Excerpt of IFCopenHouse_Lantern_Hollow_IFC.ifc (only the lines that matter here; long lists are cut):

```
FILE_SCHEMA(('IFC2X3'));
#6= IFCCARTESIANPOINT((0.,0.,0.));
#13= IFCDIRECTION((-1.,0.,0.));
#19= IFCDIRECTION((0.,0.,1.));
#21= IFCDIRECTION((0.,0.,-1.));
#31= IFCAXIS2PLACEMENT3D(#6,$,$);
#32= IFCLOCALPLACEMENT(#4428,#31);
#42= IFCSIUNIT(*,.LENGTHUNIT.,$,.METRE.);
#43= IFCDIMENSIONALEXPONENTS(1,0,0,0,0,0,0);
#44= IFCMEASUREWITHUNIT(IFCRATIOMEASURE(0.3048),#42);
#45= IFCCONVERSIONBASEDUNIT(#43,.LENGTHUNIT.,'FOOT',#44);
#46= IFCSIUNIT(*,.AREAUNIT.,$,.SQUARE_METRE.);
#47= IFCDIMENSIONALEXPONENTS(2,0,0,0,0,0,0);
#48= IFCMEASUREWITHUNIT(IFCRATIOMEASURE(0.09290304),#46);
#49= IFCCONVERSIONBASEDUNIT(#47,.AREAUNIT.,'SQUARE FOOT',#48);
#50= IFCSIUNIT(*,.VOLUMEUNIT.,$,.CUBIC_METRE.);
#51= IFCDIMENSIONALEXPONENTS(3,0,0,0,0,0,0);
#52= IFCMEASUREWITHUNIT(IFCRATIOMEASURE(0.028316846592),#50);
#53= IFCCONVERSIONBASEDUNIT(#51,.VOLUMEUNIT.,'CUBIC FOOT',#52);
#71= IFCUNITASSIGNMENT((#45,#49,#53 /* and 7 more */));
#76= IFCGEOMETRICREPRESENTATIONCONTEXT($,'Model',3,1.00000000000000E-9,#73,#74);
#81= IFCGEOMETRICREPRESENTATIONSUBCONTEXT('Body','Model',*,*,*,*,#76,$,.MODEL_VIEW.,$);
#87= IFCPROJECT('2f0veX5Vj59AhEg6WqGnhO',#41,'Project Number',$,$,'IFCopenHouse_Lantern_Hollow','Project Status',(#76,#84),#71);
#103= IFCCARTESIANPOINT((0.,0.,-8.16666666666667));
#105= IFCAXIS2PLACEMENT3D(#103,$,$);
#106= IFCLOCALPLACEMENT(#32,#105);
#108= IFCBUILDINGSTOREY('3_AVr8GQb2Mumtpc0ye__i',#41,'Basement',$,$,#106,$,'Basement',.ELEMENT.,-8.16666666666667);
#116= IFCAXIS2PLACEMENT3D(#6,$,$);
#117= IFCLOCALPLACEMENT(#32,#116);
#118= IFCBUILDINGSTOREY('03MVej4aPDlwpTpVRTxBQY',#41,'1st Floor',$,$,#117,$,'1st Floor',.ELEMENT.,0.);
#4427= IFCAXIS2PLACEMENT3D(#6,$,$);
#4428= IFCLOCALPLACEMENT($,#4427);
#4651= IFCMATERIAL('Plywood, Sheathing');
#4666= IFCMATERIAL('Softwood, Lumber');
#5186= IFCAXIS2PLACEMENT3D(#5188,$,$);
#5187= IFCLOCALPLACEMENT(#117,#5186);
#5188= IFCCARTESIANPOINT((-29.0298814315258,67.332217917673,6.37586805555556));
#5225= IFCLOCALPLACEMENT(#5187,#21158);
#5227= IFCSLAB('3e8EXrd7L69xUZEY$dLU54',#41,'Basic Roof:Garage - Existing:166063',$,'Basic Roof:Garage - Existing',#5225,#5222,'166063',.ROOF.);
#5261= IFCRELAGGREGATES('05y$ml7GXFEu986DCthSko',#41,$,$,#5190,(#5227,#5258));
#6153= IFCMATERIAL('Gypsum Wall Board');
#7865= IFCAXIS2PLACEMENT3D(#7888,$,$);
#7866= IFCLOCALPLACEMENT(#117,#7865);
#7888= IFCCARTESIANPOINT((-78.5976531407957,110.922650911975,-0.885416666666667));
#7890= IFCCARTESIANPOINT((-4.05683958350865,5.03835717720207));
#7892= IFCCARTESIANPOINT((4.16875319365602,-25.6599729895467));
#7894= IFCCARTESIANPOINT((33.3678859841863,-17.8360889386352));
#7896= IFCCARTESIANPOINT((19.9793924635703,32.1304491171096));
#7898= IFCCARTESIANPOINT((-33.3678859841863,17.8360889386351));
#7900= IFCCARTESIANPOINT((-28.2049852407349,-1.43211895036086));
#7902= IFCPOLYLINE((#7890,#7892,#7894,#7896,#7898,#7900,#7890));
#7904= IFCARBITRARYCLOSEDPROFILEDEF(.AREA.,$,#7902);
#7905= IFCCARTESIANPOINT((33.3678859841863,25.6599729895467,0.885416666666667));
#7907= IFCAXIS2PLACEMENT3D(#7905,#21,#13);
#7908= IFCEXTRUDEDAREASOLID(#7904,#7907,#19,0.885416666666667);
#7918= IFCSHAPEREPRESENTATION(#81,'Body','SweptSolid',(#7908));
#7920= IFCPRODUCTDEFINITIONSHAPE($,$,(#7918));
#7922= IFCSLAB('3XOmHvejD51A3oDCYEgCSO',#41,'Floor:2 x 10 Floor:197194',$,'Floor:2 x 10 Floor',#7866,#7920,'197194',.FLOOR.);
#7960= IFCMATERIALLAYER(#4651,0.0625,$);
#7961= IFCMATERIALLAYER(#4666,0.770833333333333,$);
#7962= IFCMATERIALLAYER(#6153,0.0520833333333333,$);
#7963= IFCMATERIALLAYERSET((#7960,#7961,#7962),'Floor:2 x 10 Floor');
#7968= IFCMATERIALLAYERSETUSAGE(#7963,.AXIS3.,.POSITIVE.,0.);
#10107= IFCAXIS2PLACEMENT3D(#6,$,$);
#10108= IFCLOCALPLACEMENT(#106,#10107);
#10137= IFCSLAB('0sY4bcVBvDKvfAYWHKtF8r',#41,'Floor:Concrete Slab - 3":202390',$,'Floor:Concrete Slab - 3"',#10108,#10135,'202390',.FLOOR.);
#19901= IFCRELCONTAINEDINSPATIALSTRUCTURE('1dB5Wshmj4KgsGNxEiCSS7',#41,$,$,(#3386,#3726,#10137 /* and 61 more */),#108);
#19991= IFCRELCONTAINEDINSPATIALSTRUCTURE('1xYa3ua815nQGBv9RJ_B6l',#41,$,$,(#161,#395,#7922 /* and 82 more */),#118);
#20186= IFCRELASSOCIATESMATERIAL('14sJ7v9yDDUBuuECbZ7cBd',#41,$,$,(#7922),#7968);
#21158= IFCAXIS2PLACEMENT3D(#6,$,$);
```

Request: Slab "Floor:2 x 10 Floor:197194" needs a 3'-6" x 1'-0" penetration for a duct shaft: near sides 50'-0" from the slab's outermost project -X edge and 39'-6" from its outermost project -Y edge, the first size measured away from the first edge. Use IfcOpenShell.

```python
import numpy as np
import ifcopenshell
import ifcopenshell.api.feature
import ifcopenshell.api.geometry
import ifcopenshell.api.root
import ifcopenshell.geom
import ifcopenshell.util.placement
import ifcopenshell.util.representation
import ifcopenshell.util.shape
import ifcopenshell.util.unit

model = ifcopenshell.open("IFCopenHouse_Lantern_Hollow_IFC.ifc")
unit_scale = ifcopenshell.util.unit.calculate_unit_scale(model)
settings = ifcopenshell.geom.settings()


def volume(element):
    """Net volume in cubic metres, openings subtracted."""
    shape = ifcopenshell.geom.create_shape(settings, element)
    return ifcopenshell.util.shape.get_volume(shape.geometry)


slab = model.by_id(7922)
before = volume(slab)

# Extent in the slab's own axes, in metres. The edges named are its -X and -Y sides.
slab_shape = ifcopenshell.geom.create_shape(settings, slab)
vertices = ifcopenshell.util.shape.get_vertices(slab_shape.geometry)
x_min, y_min, bottom = vertices.min(axis=0)
top = vertices[:, 2].max()

opening = ifcopenshell.api.root.create_entity(model, ifc_class="IfcOpeningElement", name="Duct shaft opening")
context = ifcopenshell.util.representation.get_context(model, "Model", "Body", "MODEL_VIEW")
width, depth = 1.0668, 0.3048
outline = [(0.0, 0.0), (width, 0.0), (width, depth), (0.0, depth), (0.0, 0.0)]
# Overshoot both faces by 50 mm so the cut is clean.
shape = ifcopenshell.api.geometry.add_slab_representation(
    model, context=context, depth=top - bottom + 0.1, polyline=outline
)
ifcopenshell.api.geometry.assign_representation(model, product=opening, representation=shape)

matrix = ifcopenshell.util.placement.get_local_placement(slab.ObjectPlacement)
matrix[:, 3] = matrix @ np.append(np.array([x_min + 15.24, y_min + 12.0396, bottom - 0.05]) / unit_scale, 1.0)
ifcopenshell.api.geometry.edit_object_placement(model, product=opening, matrix=matrix, is_si=False)
ifcopenshell.api.feature.add_feature(model, feature=opening, element=slab)

after = volume(slab)

print(f"slab volume {before:.3f} -> {after:.3f} m3")

model.write("IFCopenHouse_Lantern_Hollow_IFC-out.ifc")
```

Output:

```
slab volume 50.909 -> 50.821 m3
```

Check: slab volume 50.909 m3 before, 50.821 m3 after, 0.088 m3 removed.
